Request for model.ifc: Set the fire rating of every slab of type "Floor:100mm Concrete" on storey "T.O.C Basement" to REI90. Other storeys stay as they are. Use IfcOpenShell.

First a look at what the model holds.

```python
import ifcopenshell
import ifcopenshell.util.element

model = ifcopenshell.open("model.ifc")
print(model.schema)
storey = next(s for s in model.by_type("IfcBuildingStorey") if s.Name == "T.O.C Basement")
slabs = [e for e in ifcopenshell.util.element.get_decomposition(storey) if e.is_a("IfcSlab")]
seen = {}
for e in slabs:
    element_type = ifcopenshell.util.element.get_type(e)
    key = (element_type.Name if element_type != e and element_type else None, ifcopenshell.util.element.get_pset(e, "Pset_SlabCommon", "FireRating"))
    seen[key] = seen.get(key, 0) + 1
for (name, value), count in sorted(seen.items(), key=str):
    print(count, "x", name, "|", value)
```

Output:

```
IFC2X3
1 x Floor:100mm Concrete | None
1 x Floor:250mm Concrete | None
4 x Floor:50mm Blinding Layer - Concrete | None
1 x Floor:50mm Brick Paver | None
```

```python
import ifcopenshell
import ifcopenshell.api.pset
import ifcopenshell.util.element

model = ifcopenshell.open("model.ifc")

storey = next(s for s in model.by_type("IfcBuildingStorey") if s.Name == "T.O.C Basement")
slabs = [e for e in ifcopenshell.util.element.get_decomposition(storey) if e.is_a("IfcSlab")]

count = 0
for e in slabs:
    element_type = ifcopenshell.util.element.get_type(e)
    if element_type in (None, e) or element_type.Name != "Floor:100mm Concrete":
        continue
    # add_pset returns the element's existing set when there is one.
    pset = ifcopenshell.api.pset.add_pset(model, product=e, name="Pset_SlabCommon")
    ifcopenshell.api.pset.edit_pset(model, pset=pset, properties={"FireRating": "REI90"})
    count += 1

print(count, "slabs updated")

model.write("model-out.ifc")
```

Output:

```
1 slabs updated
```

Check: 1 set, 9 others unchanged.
